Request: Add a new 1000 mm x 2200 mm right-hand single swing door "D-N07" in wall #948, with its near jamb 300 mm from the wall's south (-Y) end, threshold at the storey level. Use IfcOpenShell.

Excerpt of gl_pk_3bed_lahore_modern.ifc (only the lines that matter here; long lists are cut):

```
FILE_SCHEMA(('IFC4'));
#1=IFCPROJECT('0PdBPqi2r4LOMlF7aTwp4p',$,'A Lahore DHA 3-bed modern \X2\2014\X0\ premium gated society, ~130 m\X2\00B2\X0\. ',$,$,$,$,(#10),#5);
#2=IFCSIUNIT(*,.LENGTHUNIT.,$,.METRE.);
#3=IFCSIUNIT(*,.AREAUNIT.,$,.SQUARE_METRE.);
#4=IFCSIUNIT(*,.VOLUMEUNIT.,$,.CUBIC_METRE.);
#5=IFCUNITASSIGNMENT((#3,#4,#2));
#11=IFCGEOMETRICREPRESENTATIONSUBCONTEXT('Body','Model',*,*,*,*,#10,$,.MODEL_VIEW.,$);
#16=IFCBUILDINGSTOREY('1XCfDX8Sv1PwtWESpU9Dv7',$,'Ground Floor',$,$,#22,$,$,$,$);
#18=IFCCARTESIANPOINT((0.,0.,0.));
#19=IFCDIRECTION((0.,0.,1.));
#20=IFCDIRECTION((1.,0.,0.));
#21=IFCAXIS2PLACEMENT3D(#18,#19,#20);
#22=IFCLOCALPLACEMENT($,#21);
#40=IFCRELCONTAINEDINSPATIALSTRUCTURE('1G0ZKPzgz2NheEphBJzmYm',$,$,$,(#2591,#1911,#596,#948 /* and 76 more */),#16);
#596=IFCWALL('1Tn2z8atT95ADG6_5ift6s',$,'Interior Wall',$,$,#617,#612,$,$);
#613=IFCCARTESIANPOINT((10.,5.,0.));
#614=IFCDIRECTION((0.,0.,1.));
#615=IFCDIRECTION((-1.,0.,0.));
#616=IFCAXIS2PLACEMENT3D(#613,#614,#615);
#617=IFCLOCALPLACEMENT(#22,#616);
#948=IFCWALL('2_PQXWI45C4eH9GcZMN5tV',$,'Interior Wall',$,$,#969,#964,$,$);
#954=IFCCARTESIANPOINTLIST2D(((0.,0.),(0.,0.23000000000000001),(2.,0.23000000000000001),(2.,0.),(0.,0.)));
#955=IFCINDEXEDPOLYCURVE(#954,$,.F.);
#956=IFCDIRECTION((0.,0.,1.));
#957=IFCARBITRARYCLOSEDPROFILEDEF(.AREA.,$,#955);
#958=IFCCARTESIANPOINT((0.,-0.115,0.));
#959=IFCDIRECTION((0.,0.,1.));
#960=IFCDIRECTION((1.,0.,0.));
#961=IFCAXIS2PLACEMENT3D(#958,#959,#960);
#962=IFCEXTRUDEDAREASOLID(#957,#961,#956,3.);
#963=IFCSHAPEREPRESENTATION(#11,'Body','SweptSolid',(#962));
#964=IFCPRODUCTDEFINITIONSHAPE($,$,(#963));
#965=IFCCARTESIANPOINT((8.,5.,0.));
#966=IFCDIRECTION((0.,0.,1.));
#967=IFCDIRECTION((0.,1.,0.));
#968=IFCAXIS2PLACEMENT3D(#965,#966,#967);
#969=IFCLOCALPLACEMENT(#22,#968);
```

```python
import numpy as np
import ifcopenshell
import ifcopenshell.api.feature
import ifcopenshell.api.geometry
import ifcopenshell.api.root
import ifcopenshell.api.spatial
import ifcopenshell.geom
import ifcopenshell.util.element
import ifcopenshell.util.placement
import ifcopenshell.util.representation
import ifcopenshell.util.shape
import ifcopenshell.util.unit

model = ifcopenshell.open("gl_pk_3bed_lahore_modern.ifc")
unit_scale = ifcopenshell.util.unit.calculate_unit_scale(model)
settings = ifcopenshell.geom.settings()


def volume(element):
    """Net volume in cubic metres, openings subtracted."""
    shape = ifcopenshell.geom.create_shape(settings, element)
    return ifcopenshell.util.shape.get_volume(shape.geometry)


wall = model.by_guid("2_PQXWI45C4eH9GcZMN5tV")
storey = ifcopenshell.util.element.get_container(wall, ifc_class="IfcBuildingStorey")
context = ifcopenshell.util.representation.get_context(model, "Model", "Body", "MODEL_VIEW")
before = volume(wall)

width, height, from_end, sill = 1, 2.2, 0.3, 0.0  # metres

# The wall runs along its own X axis, and the end named is its -X end.
wall_shape = ifcopenshell.geom.create_shape(settings, wall)
x, y, z = ifcopenshell.util.shape.get_vertices(wall_shape.geometry).T
start = x.min() + from_end
face, thickness = float(y.min()), float(y.max() - y.min())
wall_matrix = ifcopenshell.util.placement.get_local_placement(wall.ObjectPlacement)
level = ifcopenshell.util.placement.get_local_placement(storey.ObjectPlacement)[2, 3]


def in_wall(x, y):
    """Placement at x, y metres in the wall's axes, at sill height."""
    matrix = wall_matrix.copy()
    matrix[:, 3] = wall_matrix @ np.array([x / unit_scale, y / unit_scale, 0.0, 1.0])
    matrix[2, 3] = level + sill / unit_scale
    return matrix


# Opening: a box that overshoots both wall faces by 50 mm.
opening = ifcopenshell.api.root.create_entity(model, ifc_class="IfcOpeningElement", predefined_type="OPENING")
box = ifcopenshell.api.geometry.add_wall_representation(
    model, context=context, length=width, height=height, thickness=thickness + 0.1
)
ifcopenshell.api.geometry.assign_representation(model, product=opening, representation=box)
ifcopenshell.api.geometry.edit_object_placement(model, product=opening, matrix=in_wall(start, face - 0.05), is_si=False)
ifcopenshell.api.feature.add_feature(model, feature=opening, element=wall)

door = ifcopenshell.api.root.create_entity(model, ifc_class="IfcDoor", name="D-N07", predefined_type="DOOR")
door.OverallWidth, door.OverallHeight = width / unit_scale, height / unit_scale
door.OperationType = "SINGLE_SWING_RIGHT"
body = ifcopenshell.api.geometry.add_door_representation(
    model,
    context=context,
    overall_width=door.OverallWidth,
    overall_height=door.OverallHeight,
    operation_type="SINGLE_SWING_RIGHT",
    lining_properties={"LiningDepth": thickness / unit_scale, "ThresholdDepth": thickness / unit_scale},
)
ifcopenshell.api.geometry.assign_representation(model, product=door, representation=body)
ifcopenshell.api.spatial.assign_container(model, products=[door], relating_structure=storey)
ifcopenshell.api.feature.add_filling(model, opening=opening, element=door)

# The lining spans the wall, so the door starts at the wall face.
ifcopenshell.api.geometry.edit_object_placement(model, product=door, matrix=in_wall(start, face), is_si=False)

after = volume(wall)

print(f"wall volume {before:.3f} -> {after:.3f} m3")

model.write("gl_pk_3bed_lahore_modern_v2.ifc")
```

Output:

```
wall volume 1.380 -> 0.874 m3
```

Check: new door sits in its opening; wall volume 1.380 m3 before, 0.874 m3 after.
